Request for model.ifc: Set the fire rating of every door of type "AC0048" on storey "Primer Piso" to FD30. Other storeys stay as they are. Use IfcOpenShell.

First a look at what the model holds.

```python
import ifcopenshell
import ifcopenshell.util.element

model = ifcopenshell.open("model.ifc")
print(model.schema)
storey = next(s for s in model.by_type("IfcBuildingStorey") if s.Name == "Primer Piso")
doors = [e for e in ifcopenshell.util.element.get_decomposition(storey) if e.is_a("IfcDoor")]
seen = {}
for e in doors:
    element_type = ifcopenshell.util.element.get_type(e)
    key = (element_type.Name if element_type != e and element_type else None, ifcopenshell.util.element.get_pset(e, "Pset_DoorCommon", "FireRating"))
    seen[key] = seen.get(key, 0) + 1
for (name, value), count in sorted(seen.items(), key=str):
    print(count, "x", name, "|", value)
```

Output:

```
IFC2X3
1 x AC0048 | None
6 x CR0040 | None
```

```python
import ifcopenshell
import ifcopenshell.api.pset
import ifcopenshell.util.element

model = ifcopenshell.open("model.ifc")

storey = next(s for s in model.by_type("IfcBuildingStorey") if s.Name == "Primer Piso")
doors = [e for e in ifcopenshell.util.element.get_decomposition(storey) if e.is_a("IfcDoor")]

count = 0
for e in doors:
    element_type = ifcopenshell.util.element.get_type(e)
    if element_type in (None, e) or element_type.Name != "AC0048":
        continue
    # add_pset returns the element's existing set when there is one.
    pset = ifcopenshell.api.pset.add_pset(model, product=e, name="Pset_DoorCommon")
    ifcopenshell.api.pset.edit_pset(model, pset=pset, properties={"FireRating": "FD30"})
    count += 1

print(count, "doors updated")

model.write("model_edited.ifc")
```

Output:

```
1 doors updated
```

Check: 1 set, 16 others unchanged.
